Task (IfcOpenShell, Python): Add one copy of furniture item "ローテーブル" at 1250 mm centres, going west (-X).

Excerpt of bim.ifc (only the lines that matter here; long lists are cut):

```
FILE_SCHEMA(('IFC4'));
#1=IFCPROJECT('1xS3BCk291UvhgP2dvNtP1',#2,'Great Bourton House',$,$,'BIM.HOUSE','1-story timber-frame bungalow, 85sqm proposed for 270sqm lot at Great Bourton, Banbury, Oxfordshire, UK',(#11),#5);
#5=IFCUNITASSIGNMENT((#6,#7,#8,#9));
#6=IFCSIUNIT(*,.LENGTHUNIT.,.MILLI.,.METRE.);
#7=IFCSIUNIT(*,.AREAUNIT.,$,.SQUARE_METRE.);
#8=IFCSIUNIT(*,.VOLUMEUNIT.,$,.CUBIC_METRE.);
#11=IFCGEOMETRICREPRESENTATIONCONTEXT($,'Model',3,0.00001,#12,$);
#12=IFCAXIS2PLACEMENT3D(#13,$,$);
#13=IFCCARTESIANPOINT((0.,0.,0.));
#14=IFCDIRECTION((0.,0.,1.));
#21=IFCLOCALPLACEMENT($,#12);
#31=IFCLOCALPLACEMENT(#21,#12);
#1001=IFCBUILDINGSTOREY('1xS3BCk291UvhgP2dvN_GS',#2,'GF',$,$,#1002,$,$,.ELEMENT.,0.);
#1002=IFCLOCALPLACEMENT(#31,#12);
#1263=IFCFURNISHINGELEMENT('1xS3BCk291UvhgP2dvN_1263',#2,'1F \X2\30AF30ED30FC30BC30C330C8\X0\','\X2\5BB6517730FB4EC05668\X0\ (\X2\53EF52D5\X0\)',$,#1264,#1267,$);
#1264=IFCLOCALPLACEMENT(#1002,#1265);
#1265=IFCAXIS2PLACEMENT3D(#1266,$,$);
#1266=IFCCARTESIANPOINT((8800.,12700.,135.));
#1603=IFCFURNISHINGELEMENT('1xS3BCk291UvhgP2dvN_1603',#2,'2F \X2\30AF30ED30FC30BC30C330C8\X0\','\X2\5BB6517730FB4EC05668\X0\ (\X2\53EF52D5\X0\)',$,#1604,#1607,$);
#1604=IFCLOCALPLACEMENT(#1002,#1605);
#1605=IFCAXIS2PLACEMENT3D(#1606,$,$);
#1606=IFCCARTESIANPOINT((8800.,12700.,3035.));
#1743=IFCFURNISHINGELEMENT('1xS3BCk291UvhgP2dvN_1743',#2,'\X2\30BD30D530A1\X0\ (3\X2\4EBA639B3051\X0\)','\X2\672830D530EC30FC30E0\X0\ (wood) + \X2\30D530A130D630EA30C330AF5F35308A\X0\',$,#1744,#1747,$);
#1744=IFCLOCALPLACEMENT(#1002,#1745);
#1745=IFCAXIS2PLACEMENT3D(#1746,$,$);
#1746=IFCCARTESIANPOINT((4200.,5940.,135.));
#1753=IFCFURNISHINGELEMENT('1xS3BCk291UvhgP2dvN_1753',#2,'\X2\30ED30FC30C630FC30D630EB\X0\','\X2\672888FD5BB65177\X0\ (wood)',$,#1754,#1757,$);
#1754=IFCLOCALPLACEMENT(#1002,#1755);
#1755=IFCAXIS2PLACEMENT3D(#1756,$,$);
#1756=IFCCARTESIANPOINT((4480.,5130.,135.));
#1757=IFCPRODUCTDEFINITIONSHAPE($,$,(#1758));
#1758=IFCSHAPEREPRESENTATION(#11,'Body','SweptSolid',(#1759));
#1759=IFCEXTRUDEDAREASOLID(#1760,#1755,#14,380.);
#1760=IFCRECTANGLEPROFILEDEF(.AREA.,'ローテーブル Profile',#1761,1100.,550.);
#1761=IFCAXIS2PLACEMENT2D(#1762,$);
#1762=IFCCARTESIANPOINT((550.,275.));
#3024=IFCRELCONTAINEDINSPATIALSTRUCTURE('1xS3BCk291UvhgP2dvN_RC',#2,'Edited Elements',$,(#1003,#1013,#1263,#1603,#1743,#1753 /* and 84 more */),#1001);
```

```python
import numpy as np
import ifcopenshell
import ifcopenshell.api.geometry
import ifcopenshell.api.root
import ifcopenshell.util.element
import ifcopenshell.util.placement
import ifcopenshell.util.unit

model = ifcopenshell.open("bim.ifc")
unit_scale = ifcopenshell.util.unit.calculate_unit_scale(model)


def reuse_history(source, copy):
    """copy_class also copies each property set's owner history, people and application; keep the originals."""
    for rel in copy.IsDefinedBy:
        if rel.is_a("IfcRelDefinesByProperties") and (history := rel.RelatingPropertyDefinition.OwnerHistory):
            rel.RelatingPropertyDefinition.OwnerHistory = source.OwnerHistory
            ifcopenshell.util.element.remove_deep2(model, history)


source = model.by_guid("1xS3BCk291UvhgP2dvN_1753")
base = ifcopenshell.util.placement.get_local_placement(source.ObjectPlacement)
step = np.array([-1.0, 0.0, 0.0]) * 1.25 / unit_scale

for i in range(1, 2):
    copy = ifcopenshell.api.root.copy_class(model, product=source)
    copy.Representation = ifcopenshell.util.element.copy_deep(
        model, source.Representation, exclude=["IfcGeometricRepresentationContext", "IfcRepresentationMap"]
    )
    reuse_history(source, copy)
    matrix = base.copy()
    matrix[:3, 3] += i * step
    print("added at", matrix[:3, 3].round(3) + 0.0)
    ifcopenshell.api.geometry.edit_object_placement(model, product=copy, matrix=matrix, is_si=False)

model.write("bim_updated.ifc")
```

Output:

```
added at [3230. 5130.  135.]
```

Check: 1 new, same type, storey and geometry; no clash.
